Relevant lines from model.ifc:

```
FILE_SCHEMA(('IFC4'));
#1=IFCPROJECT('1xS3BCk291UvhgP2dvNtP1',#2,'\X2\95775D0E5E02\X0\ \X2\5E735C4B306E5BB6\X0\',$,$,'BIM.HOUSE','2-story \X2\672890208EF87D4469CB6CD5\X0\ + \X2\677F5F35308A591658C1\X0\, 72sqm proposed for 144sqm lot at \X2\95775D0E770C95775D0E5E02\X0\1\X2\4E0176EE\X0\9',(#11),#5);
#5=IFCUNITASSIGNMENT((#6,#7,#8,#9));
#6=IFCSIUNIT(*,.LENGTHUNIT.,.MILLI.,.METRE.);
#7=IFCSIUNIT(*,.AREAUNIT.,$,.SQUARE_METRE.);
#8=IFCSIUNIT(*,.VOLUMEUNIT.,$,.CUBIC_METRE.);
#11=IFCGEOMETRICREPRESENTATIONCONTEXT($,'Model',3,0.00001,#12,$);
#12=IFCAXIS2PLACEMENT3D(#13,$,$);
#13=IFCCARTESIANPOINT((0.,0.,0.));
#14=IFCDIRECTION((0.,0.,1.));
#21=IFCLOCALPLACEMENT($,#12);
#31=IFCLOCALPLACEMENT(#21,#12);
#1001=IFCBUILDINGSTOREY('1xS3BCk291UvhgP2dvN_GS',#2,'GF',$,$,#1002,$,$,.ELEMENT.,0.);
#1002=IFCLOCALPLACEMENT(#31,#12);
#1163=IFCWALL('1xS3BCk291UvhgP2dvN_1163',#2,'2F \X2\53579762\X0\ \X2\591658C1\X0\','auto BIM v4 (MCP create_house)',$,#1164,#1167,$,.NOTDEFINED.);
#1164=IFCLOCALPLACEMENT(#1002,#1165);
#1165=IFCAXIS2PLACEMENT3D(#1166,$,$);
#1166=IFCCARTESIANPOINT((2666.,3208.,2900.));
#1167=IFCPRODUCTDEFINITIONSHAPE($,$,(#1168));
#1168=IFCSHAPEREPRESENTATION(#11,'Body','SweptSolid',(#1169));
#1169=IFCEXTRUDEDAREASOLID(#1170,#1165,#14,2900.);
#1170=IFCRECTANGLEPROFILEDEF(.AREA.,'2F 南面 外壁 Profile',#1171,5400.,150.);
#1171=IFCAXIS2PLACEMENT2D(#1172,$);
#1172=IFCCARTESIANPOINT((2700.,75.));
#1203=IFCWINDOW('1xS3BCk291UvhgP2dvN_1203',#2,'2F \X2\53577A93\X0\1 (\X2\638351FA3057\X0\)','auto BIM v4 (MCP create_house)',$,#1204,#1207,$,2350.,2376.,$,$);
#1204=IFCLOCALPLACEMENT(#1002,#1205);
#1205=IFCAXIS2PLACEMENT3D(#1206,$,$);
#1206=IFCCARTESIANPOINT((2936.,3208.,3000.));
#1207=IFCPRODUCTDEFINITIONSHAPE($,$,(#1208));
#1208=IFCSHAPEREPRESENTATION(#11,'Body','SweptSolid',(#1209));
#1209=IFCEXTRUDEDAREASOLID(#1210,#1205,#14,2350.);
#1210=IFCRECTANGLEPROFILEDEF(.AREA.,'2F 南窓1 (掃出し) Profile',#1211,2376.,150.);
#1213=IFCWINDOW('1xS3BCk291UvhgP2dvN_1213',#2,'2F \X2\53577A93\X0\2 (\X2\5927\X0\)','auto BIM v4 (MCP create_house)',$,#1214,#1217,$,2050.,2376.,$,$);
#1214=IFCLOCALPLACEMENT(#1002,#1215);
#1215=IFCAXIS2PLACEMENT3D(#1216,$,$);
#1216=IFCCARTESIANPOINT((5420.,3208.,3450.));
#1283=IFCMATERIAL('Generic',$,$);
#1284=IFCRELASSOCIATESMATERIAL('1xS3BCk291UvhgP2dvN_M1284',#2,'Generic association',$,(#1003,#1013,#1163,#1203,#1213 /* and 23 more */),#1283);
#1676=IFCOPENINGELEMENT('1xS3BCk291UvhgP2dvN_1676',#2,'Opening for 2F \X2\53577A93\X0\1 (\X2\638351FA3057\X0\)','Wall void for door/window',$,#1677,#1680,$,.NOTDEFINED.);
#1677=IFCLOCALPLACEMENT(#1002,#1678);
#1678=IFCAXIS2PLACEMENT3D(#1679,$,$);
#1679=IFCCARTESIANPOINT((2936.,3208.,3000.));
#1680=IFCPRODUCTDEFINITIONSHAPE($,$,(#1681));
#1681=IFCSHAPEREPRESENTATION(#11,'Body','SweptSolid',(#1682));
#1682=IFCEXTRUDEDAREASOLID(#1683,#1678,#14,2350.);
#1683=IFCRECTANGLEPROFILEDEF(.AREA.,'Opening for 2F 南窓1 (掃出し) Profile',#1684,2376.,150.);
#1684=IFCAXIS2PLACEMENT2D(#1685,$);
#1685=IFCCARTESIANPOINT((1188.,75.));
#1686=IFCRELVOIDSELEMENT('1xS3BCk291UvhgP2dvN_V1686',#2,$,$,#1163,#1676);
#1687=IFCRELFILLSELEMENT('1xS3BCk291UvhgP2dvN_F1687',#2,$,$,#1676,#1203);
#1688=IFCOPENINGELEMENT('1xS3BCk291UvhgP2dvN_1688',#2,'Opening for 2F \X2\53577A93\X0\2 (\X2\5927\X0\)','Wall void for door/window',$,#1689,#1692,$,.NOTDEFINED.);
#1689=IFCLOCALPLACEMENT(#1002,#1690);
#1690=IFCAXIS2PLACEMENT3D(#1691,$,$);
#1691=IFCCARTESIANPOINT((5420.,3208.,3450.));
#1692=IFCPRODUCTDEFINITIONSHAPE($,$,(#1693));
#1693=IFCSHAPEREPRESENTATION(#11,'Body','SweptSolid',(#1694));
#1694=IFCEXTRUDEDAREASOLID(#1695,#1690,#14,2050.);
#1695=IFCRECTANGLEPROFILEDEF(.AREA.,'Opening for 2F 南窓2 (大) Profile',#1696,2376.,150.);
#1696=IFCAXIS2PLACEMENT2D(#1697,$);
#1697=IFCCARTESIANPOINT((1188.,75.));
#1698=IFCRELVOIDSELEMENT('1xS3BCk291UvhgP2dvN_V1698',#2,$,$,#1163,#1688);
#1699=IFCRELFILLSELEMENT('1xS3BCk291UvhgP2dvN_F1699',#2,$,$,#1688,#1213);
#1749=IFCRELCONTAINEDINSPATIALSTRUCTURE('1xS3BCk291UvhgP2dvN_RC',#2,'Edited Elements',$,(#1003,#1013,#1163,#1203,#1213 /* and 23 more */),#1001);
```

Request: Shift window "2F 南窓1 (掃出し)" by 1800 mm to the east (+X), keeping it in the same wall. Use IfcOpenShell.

```python
import ifcopenshell
import ifcopenshell.api.geometry
import ifcopenshell.util.placement
import ifcopenshell.util.unit

model = ifcopenshell.open("model.ifc")
unit_scale = ifcopenshell.util.unit.calculate_unit_scale(model)

window = model.by_guid("1xS3BCk291UvhgP2dvN_1203")
opening = window.FillsVoids[0].RelatingOpeningElement
wall = opening.VoidsElements[0].RelatingBuildingElement

wall_matrix = ifcopenshell.util.placement.get_local_placement(wall.ObjectPlacement)
shift = wall_matrix[:3, 0] * 1.8 / unit_scale
before = ifcopenshell.util.placement.get_local_placement(window.ObjectPlacement)[:3, 3].copy()

# The window is not placed relative to its opening, so move both.
for product in (opening, window):
    matrix = ifcopenshell.util.placement.get_local_placement(product.ObjectPlacement)
    matrix[:3, 3] += shift
    ifcopenshell.api.geometry.edit_object_placement(model, product=product, matrix=matrix, is_si=False)

after = ifcopenshell.util.placement.get_local_placement(window.ObjectPlacement)[:3, 3]
print("window moved by", (after - before).round(3) + 0.0)

model.write("model_edited.ifc")
```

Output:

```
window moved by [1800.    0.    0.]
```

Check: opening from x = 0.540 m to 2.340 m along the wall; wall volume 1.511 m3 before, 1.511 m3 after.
